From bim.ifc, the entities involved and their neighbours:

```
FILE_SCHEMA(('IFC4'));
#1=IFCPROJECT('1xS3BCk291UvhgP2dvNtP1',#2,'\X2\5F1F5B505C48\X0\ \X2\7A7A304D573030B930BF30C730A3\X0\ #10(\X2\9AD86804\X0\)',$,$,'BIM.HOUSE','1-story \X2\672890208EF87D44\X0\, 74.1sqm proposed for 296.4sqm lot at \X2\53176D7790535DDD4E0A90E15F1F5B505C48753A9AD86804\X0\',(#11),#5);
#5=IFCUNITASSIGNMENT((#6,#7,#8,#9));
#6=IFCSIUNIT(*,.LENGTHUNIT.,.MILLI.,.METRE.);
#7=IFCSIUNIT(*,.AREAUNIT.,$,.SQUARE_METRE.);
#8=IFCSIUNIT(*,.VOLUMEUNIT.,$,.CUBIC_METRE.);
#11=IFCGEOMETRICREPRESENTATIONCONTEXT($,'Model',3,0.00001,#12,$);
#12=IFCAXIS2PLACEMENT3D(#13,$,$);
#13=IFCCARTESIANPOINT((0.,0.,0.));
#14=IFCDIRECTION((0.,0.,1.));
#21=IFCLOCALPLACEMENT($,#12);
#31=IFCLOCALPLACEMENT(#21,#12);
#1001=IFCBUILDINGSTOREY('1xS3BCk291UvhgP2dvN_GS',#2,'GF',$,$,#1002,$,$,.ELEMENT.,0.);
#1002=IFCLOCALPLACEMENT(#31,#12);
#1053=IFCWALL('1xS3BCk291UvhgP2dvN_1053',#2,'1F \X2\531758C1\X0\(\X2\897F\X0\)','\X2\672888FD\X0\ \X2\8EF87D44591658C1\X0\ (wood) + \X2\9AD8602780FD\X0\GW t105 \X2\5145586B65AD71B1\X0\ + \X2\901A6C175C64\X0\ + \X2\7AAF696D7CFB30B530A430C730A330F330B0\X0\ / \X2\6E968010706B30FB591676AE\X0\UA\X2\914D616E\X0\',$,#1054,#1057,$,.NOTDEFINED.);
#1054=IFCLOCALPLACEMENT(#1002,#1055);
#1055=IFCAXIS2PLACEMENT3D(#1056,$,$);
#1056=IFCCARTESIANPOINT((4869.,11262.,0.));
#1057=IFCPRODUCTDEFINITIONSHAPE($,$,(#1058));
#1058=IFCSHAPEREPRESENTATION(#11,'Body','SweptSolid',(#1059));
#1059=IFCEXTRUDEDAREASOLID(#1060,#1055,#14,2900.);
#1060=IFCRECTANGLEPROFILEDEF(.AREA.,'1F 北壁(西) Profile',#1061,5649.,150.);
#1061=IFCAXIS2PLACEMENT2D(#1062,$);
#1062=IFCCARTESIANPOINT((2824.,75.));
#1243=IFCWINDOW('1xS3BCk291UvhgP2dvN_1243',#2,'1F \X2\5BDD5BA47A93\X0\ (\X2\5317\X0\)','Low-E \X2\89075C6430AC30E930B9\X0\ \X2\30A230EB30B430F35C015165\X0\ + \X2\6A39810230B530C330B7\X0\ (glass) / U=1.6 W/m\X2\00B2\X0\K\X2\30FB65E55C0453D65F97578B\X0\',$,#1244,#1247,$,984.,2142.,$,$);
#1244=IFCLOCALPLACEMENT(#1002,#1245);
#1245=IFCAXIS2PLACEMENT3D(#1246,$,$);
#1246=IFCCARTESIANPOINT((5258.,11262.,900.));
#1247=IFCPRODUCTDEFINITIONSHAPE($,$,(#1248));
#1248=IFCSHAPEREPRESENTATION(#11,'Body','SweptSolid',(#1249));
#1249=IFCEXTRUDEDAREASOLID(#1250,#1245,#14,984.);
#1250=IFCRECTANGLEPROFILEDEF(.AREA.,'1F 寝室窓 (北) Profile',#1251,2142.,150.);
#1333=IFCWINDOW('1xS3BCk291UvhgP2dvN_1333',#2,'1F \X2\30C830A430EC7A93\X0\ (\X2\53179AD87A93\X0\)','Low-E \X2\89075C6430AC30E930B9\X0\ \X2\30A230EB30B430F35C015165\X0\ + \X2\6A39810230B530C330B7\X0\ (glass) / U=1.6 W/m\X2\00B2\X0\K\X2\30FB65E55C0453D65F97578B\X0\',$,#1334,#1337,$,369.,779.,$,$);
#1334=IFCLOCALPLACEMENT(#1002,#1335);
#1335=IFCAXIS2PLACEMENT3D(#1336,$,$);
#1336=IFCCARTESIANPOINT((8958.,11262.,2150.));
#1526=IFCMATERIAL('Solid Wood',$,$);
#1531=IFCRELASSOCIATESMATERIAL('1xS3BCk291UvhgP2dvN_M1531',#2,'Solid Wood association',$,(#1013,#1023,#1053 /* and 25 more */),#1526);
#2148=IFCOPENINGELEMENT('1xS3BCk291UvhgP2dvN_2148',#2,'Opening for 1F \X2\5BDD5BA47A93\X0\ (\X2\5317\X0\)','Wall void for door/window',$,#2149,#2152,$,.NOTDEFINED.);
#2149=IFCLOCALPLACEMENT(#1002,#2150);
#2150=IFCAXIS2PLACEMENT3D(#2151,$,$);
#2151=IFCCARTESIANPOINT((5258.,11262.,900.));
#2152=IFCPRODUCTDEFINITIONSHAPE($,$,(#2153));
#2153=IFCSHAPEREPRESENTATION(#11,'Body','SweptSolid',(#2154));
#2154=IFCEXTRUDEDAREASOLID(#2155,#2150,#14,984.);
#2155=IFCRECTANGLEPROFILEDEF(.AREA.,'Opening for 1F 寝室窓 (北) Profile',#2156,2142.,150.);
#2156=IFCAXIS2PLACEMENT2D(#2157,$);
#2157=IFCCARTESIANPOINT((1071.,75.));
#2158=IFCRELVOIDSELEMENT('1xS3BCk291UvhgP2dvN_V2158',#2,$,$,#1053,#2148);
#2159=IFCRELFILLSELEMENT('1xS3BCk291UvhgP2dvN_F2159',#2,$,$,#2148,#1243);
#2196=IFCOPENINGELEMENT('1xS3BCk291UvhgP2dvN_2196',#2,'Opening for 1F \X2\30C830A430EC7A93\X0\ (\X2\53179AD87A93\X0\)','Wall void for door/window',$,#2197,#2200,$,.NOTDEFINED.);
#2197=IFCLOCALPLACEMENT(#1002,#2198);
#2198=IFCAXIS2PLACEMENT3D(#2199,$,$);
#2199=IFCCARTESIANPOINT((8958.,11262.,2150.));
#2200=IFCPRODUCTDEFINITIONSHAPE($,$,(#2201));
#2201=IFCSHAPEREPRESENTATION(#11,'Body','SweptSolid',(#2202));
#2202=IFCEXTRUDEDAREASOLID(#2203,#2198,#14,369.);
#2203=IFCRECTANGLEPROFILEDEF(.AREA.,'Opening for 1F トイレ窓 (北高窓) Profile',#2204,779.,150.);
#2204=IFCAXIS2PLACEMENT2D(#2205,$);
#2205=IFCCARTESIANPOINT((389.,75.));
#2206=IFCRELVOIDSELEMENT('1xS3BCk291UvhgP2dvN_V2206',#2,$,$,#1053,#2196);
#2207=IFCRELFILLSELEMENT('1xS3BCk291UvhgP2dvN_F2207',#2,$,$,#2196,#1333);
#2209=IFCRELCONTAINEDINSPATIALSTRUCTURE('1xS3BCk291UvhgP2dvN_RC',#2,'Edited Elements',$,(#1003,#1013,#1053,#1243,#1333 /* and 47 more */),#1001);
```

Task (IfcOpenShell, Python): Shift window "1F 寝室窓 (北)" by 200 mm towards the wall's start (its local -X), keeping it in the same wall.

```python
import ifcopenshell
import ifcopenshell.api.geometry
import ifcopenshell.util.placement

model = ifcopenshell.open("bim.ifc")

window = model.by_guid("1xS3BCk291UvhgP2dvN_1243")
opening = window.FillsVoids[0].RelatingOpeningElement
wall = opening.VoidsElements[0].RelatingBuildingElement

wall_matrix = ifcopenshell.util.placement.get_local_placement(wall.ObjectPlacement)
shift = wall_matrix[:3, 0] * -200.0
before = ifcopenshell.util.placement.get_local_placement(window.ObjectPlacement)[:3, 3].copy()

# The window is not placed relative to its opening, so move both.
for product in (opening, window):
    matrix = ifcopenshell.util.placement.get_local_placement(product.ObjectPlacement)
    matrix[:3, 3] += shift
    ifcopenshell.api.geometry.edit_object_placement(model, product=product, matrix=matrix, is_si=False)

after = ifcopenshell.util.placement.get_local_placement(window.ObjectPlacement)[:3, 3]
print("window moved by", (after - before).round(3) + 0.0)

model.write("bim_edited.ifc")
```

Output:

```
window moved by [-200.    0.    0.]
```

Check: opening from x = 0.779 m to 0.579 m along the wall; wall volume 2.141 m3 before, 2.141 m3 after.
